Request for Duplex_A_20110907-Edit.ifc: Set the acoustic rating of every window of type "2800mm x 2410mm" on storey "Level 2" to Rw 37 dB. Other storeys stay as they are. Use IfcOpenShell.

First a look at what the model holds.

```python
import ifcopenshell
import ifcopenshell.util.element

model = ifcopenshell.open("Duplex_A_20110907-Edit.ifc")
print(model.schema)
storey = next(s for s in model.by_type("IfcBuildingStorey") if s.Name == "Level 2")
windows = [e for e in ifcopenshell.util.element.get_decomposition(storey) if e.is_a("IfcWindow")]
seen = {}
for e in windows:
    element_type = ifcopenshell.util.element.get_type(e)
    key = (element_type.Name if element_type != e and element_type else None, ifcopenshell.util.element.get_pset(e, "Pset_WindowCommon", "AcousticRating"))
    seen[key] = seen.get(key, 0) + 1
for (name, value), count in sorted(seen.items(), key=str):
    print(count, "x", name, "|", value)
```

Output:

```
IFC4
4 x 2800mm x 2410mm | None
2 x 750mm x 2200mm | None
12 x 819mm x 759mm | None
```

```python
import ifcopenshell
import ifcopenshell.api.pset
import ifcopenshell.util.element

model = ifcopenshell.open("Duplex_A_20110907-Edit.ifc")

storey = next(s for s in model.by_type("IfcBuildingStorey") if s.Name == "Level 2")
windows = [e for e in ifcopenshell.util.element.get_decomposition(storey) if e.is_a("IfcWindow")]

count = 0
for e in windows:
    element_type = ifcopenshell.util.element.get_type(e)
    if element_type in (None, e) or element_type.Name != "2800mm x 2410mm":
        continue
    # add_pset returns the element's existing set when there is one.
    pset = ifcopenshell.api.pset.add_pset(model, product=e, name="Pset_WindowCommon")
    ifcopenshell.api.pset.edit_pset(model, pset=pset, properties={"AcousticRating": "Rw 37 dB"})
    count += 1

print(count, "windows updated")

model.write("Duplex_A_20110907-Edit-out.ifc")
```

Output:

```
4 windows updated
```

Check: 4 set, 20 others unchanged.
